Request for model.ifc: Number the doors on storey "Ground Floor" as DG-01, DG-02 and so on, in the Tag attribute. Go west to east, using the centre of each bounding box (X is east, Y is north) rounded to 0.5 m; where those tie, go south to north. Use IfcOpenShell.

First a look at what the model holds.

```python
import ifcopenshell
import ifcopenshell.util.element
import ifcopenshell.util.placement

model = ifcopenshell.open("model.ifc")
print(model.schema)
storey = next(s for s in model.by_type("IfcBuildingStorey") if s.Name == "Ground Floor")
doors = [e for e in ifcopenshell.util.element.get_decomposition(storey) if e.is_a("IfcDoor")]
for e in sorted(doors, key=lambda e: e.id()):
    origin = ifcopenshell.util.placement.get_local_placement(e.ObjectPlacement)[:3, 3]
    print(e.id(), e.Tag, e.Name, origin.round(2) + 0.0, sep=" | ")
```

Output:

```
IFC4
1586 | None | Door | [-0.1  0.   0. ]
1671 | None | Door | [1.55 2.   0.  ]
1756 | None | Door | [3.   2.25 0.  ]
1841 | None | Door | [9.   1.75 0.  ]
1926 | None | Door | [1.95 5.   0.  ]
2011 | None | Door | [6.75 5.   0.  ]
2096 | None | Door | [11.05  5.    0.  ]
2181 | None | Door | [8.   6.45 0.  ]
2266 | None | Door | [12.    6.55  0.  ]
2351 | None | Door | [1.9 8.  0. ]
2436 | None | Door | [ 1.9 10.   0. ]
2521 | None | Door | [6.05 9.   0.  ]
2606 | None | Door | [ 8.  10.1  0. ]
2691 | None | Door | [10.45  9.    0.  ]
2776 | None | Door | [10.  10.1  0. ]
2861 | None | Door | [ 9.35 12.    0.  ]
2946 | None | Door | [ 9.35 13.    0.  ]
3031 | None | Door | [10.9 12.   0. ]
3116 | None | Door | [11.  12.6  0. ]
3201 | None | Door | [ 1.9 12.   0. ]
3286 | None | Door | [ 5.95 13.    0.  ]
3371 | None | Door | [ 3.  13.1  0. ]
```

```python
import ifcopenshell
import ifcopenshell.geom
import ifcopenshell.util.element
import ifcopenshell.util.shape

model = ifcopenshell.open("model.ifc")
settings = ifcopenshell.geom.settings()
settings.set("use-world-coords", True)


def centre(element):
    shape = ifcopenshell.geom.create_shape(settings, element)
    return ifcopenshell.util.shape.get_bbox_centroid(shape.geometry)


storey = next(s for s in model.by_type("IfcBuildingStorey") if s.Name == "Ground Floor")
doors = [e for e in ifcopenshell.util.element.get_decomposition(storey) if e.is_a("IfcDoor")]

# Insertion points can sit at a corner or the storey origin, so sort by the geometry (in metres).
centres = {e: centre(e) for e in doors}
doors.sort(key=lambda e: (round(centres[e][0] / 0.5), centres[e][1]))

for i, e in enumerate(doors, start=1):
    number = f"DG-{i:02d}"
    e.Tag = number
    print(e.id(), number)

model.write("model_edited.ifc")
```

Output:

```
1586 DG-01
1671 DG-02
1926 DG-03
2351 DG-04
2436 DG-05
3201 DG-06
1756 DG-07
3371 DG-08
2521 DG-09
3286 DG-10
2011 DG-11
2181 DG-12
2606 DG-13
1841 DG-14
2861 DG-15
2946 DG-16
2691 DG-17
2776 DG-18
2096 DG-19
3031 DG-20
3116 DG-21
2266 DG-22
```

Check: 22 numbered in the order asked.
